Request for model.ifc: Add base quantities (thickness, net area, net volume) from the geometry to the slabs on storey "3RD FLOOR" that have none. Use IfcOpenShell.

First a look at what the model holds.

```python
import ifcopenshell
import ifcopenshell.util.element
import ifcopenshell.util.unit

model = ifcopenshell.open("model.ifc")
print(model.schema)
for unit_type in ("LENGTHUNIT", "AREAUNIT", "VOLUMEUNIT"):
    print(unit_type, ifcopenshell.util.unit.calculate_unit_scale(model, unit_type))
storey = next(s for s in model.by_type("IfcBuildingStorey") if s.Name == "3RD FLOOR")
slabs = [e for e in ifcopenshell.util.element.get_decomposition(storey) if e.is_a("IfcSlab")]
for e in sorted(slabs, key=lambda e: e.id()):
    print(e.id(), e.is_a(), e.Name, list(ifcopenshell.util.element.get_psets(e, qtos_only=True)), sep=" | ")
```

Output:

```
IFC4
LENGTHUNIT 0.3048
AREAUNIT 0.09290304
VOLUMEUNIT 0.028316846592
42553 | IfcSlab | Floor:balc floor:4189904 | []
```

```python
import ifcopenshell
import ifcopenshell.api.pset
import ifcopenshell.geom
import ifcopenshell.util.element
import ifcopenshell.util.shape
import ifcopenshell.util.unit

model = ifcopenshell.open("model.ifc")
unit_scale = ifcopenshell.util.unit.calculate_unit_scale(model)
area_scale = ifcopenshell.util.unit.calculate_unit_scale(model, "AREAUNIT")
volume_scale = ifcopenshell.util.unit.calculate_unit_scale(model, "VOLUMEUNIT")
settings = ifcopenshell.geom.settings()

storey = next(s for s in model.by_type("IfcBuildingStorey") if s.Name == "3RD FLOOR")
slabs = [e for e in ifcopenshell.util.element.get_decomposition(storey) if e.is_a("IfcSlab")]

for e in sorted(slabs, key=lambda e: e.id()):
    if ifcopenshell.util.element.get_psets(e, qtos_only=True, should_inherit=False):
        continue
    # Geometry comes back in metres, in the element's own axes.
    shape = ifcopenshell.geom.create_shape(settings, e)
    values = {
        "Width": ifcopenshell.util.shape.get_z(shape.geometry) / unit_scale,
        "NetArea": ifcopenshell.util.shape.get_footprint_area(shape.geometry) / area_scale,
        "NetVolume": ifcopenshell.util.shape.get_volume(shape.geometry) / volume_scale,
    }
    qto = ifcopenshell.api.pset.add_qto(model, product=e, name="Qto_SlabBaseQuantities")
    ifcopenshell.api.pset.edit_qto(model, qto=qto, properties=values)
    print(e.id(), {k: round(v, 3) for k, v in values.items()})

model.write("model_v2.ifc")
```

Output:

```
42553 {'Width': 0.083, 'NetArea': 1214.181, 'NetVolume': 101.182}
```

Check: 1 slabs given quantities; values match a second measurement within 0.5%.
